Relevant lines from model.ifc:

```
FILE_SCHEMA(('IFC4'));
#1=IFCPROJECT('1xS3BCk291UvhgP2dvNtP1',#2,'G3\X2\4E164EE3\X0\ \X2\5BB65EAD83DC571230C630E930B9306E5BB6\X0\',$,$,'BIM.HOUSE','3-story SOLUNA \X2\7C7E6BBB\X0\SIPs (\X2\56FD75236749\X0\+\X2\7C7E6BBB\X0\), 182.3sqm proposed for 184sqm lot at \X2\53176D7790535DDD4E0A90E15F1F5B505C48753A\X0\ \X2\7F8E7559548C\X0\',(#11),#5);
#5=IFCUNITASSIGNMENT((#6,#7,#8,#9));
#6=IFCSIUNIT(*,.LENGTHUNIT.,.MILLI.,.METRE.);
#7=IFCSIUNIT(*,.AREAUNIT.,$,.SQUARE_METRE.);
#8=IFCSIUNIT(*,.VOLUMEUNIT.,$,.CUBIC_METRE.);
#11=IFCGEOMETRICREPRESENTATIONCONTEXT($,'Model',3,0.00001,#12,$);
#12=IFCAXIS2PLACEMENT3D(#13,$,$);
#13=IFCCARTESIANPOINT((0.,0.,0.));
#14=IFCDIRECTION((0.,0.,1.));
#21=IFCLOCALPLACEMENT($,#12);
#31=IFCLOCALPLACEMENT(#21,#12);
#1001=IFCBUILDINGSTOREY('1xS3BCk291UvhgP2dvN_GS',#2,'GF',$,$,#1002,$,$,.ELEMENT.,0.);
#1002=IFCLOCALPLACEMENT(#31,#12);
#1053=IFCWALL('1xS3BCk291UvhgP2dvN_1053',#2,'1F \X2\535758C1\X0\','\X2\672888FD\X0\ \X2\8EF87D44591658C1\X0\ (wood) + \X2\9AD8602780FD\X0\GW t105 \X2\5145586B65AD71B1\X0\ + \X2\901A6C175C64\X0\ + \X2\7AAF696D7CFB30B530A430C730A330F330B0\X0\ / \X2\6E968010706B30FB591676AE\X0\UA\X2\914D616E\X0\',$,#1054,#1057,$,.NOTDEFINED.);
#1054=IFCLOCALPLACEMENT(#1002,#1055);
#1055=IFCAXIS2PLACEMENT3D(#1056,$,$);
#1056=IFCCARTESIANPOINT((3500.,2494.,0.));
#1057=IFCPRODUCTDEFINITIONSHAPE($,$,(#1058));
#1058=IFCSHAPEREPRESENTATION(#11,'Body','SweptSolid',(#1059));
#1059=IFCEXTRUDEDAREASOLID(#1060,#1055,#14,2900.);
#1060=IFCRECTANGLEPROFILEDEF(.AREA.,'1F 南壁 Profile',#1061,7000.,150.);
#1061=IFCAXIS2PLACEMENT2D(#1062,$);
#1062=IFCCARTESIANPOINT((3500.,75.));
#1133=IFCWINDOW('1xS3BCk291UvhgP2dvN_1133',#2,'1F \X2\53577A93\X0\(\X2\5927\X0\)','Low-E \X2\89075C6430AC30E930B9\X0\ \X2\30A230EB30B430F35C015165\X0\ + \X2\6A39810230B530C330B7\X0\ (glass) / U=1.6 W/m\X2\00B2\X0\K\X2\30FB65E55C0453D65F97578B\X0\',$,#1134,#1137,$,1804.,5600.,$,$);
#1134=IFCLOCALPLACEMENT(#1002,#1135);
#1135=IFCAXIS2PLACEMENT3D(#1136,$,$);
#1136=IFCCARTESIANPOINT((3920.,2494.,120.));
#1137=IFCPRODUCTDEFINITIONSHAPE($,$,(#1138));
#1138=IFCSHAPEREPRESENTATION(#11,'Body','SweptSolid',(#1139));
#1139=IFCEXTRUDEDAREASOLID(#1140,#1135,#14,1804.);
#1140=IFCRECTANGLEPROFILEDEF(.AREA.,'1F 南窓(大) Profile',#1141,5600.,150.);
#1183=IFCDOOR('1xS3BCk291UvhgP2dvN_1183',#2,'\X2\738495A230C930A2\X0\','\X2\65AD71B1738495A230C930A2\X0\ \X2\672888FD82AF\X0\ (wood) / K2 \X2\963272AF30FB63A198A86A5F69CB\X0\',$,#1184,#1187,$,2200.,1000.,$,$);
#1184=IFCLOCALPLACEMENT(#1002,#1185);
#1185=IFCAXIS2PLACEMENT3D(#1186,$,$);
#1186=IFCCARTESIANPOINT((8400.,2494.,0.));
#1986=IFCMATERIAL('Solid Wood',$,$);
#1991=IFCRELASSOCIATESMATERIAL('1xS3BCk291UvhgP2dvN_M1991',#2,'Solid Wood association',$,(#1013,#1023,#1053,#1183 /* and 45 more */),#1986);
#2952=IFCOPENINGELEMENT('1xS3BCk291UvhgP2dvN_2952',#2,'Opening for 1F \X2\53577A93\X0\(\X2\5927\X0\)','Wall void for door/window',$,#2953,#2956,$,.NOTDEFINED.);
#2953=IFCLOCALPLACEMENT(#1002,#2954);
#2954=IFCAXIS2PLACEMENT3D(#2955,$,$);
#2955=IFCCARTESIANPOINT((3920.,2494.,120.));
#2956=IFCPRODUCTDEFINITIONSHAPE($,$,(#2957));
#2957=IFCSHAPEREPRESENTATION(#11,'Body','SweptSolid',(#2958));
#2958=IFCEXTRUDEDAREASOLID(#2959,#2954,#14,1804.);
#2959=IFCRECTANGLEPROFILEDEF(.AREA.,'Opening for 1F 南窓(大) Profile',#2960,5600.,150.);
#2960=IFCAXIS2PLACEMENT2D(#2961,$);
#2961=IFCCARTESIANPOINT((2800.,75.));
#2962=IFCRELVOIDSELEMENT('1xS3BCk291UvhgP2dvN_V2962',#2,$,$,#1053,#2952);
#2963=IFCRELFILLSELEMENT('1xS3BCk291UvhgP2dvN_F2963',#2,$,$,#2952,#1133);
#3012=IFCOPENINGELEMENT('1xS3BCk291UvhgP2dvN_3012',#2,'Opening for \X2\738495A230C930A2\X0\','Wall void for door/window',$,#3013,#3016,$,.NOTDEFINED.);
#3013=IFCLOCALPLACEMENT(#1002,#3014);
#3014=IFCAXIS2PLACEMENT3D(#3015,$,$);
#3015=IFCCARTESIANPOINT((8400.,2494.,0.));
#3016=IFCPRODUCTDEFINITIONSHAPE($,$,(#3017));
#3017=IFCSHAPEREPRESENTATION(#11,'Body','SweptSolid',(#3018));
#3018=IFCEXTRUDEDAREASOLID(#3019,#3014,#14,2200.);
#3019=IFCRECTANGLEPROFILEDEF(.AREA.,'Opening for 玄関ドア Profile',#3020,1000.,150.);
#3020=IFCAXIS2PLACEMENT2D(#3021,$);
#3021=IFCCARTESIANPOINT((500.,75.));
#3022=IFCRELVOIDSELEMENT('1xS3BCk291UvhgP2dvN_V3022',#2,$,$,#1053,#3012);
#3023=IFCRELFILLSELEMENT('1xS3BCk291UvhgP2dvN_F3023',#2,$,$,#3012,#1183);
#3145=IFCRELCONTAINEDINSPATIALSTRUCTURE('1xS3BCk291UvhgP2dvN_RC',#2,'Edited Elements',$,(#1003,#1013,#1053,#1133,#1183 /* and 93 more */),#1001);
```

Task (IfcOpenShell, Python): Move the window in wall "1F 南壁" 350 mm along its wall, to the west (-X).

```python
import ifcopenshell
import ifcopenshell.api.geometry
import ifcopenshell.util.placement

model = ifcopenshell.open("model.ifc")

window = model.by_guid("1xS3BCk291UvhgP2dvN_1133")
opening = window.FillsVoids[0].RelatingOpeningElement
wall = opening.VoidsElements[0].RelatingBuildingElement

wall_matrix = ifcopenshell.util.placement.get_local_placement(wall.ObjectPlacement)
shift = wall_matrix[:3, 0] * -350.0
before = ifcopenshell.util.placement.get_local_placement(window.ObjectPlacement)[:3, 3].copy()

# The window is not placed relative to its opening, so move both.
for product in (opening, window):
    matrix = ifcopenshell.util.placement.get_local_placement(product.ObjectPlacement)
    matrix[:3, 3] += shift
    ifcopenshell.api.geometry.edit_object_placement(model, product=product, matrix=matrix, is_si=False)

after = ifcopenshell.util.placement.get_local_placement(window.ObjectPlacement)[:3, 3]
print("window moved by", (after - before).round(3) + 0.0)

model.write("model_v2.ifc")
```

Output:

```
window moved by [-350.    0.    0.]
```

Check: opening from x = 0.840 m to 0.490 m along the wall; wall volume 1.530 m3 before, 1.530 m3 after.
